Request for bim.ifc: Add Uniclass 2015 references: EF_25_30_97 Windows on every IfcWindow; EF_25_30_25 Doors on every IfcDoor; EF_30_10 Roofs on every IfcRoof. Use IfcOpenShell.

First a look at what the model holds.

```python
import ifcopenshell

model = ifcopenshell.open("bim.ifc")
print(model.schema)
print("classifications:", [c.Name for c in model.by_type("IfcClassification")])
for ifc_class in ("IfcDoor", "IfcRoof", "IfcStair", "IfcWall", "IfcWindow"):
    print(ifc_class, len(model.by_type(ifc_class)))
```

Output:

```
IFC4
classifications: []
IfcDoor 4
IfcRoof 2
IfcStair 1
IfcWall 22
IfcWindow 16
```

```python
import ifcopenshell
import ifcopenshell.api.classification

model = ifcopenshell.open("bim.ifc")

system = ifcopenshell.api.classification.add_classification(model, classification="Uniclass 2015")

codes = {
    "IfcWindow": ("EF_25_30_97", "Windows"),
    "IfcDoor": ("EF_25_30_25", "Doors"),
    "IfcRoof": ("EF_30_10", "Roofs"),
}
for ifc_class, (code, name) in codes.items():
    products = model.by_type(ifc_class)
    ifcopenshell.api.classification.add_reference(
        model, products=products, classification=system, identification=code, name=name
    )
    print(code, len(products))

model.write("bim-out.ifc")
```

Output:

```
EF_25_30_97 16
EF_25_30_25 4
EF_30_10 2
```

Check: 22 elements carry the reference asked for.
